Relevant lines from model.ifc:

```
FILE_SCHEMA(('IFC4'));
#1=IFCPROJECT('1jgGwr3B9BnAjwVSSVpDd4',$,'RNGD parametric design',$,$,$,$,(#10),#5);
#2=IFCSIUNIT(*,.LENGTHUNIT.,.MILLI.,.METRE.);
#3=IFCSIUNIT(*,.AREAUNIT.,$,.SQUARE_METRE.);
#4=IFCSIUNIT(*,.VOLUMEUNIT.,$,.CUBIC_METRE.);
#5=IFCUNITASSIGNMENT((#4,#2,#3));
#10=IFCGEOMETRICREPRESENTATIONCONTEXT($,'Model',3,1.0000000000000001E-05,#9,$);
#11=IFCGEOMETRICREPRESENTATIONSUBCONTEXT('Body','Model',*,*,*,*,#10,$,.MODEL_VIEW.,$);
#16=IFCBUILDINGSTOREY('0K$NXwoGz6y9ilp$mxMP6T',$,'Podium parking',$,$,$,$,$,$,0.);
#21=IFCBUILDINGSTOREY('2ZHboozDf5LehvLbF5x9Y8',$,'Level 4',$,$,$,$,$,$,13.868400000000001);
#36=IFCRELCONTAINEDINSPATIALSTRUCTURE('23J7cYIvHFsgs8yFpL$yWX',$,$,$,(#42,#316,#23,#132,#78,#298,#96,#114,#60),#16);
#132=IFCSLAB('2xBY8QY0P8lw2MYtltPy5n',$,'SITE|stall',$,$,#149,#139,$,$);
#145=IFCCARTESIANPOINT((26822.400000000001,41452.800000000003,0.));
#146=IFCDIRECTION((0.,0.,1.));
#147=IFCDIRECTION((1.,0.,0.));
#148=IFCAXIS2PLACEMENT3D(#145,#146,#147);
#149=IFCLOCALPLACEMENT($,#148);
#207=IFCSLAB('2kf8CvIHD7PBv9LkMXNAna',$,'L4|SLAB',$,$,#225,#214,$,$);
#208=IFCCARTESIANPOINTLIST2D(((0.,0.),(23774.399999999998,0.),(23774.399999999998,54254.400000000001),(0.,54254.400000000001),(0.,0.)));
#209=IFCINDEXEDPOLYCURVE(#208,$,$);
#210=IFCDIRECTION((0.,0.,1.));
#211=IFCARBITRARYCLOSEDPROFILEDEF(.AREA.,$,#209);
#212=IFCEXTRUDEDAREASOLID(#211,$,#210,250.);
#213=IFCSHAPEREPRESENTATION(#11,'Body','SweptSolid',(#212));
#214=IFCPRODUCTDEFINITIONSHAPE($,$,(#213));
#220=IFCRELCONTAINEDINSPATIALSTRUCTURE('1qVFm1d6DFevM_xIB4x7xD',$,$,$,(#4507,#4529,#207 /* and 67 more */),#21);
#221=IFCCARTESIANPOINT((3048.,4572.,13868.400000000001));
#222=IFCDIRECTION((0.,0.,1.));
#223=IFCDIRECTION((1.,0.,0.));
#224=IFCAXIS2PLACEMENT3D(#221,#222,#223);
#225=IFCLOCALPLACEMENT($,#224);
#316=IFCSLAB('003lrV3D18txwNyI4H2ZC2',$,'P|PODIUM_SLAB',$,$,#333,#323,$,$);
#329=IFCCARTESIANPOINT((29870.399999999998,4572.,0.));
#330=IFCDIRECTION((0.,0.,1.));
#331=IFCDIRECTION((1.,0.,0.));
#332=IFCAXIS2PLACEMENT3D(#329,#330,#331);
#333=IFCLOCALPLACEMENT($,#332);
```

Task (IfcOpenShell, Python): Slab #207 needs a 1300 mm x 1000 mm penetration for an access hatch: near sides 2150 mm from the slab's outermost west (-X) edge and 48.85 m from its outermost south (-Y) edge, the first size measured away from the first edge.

```python
import numpy as np
import ifcopenshell
import ifcopenshell.api.feature
import ifcopenshell.api.geometry
import ifcopenshell.api.root
import ifcopenshell.geom
import ifcopenshell.util.placement
import ifcopenshell.util.representation
import ifcopenshell.util.shape
import ifcopenshell.util.unit

model = ifcopenshell.open("model.ifc")
unit_scale = ifcopenshell.util.unit.calculate_unit_scale(model)
settings = ifcopenshell.geom.settings()


def volume(element):
    """Net volume in cubic metres, openings subtracted."""
    shape = ifcopenshell.geom.create_shape(settings, element)
    return ifcopenshell.util.shape.get_volume(shape.geometry)


slab = model.by_guid("2kf8CvIHD7PBv9LkMXNAna")
before = volume(slab)

# Extent in the slab's own axes, in metres. The edges named are its -X and -Y sides.
slab_shape = ifcopenshell.geom.create_shape(settings, slab)
vertices = ifcopenshell.util.shape.get_vertices(slab_shape.geometry)
x_min, y_min, bottom = vertices.min(axis=0)
top = vertices[:, 2].max()

opening = ifcopenshell.api.root.create_entity(model, ifc_class="IfcOpeningElement", name="Access hatch opening", predefined_type="OPENING")
context = ifcopenshell.util.representation.get_context(model, "Model", "Body", "MODEL_VIEW")
width, depth = 1.3, 1
outline = [(0.0, 0.0), (width, 0.0), (width, depth), (0.0, depth), (0.0, 0.0)]
# Overshoot both faces by 50 mm so the cut is clean.
shape = ifcopenshell.api.geometry.add_slab_representation(
    model, context=context, depth=top - bottom + 0.1, polyline=outline
)
ifcopenshell.api.geometry.assign_representation(model, product=opening, representation=shape)

matrix = ifcopenshell.util.placement.get_local_placement(slab.ObjectPlacement)
matrix[:, 3] = matrix @ np.append(np.array([x_min + 2.15, y_min + 48.85, bottom - 0.05]) / unit_scale, 1.0)
ifcopenshell.api.geometry.edit_object_placement(model, product=opening, matrix=matrix, is_si=False)
ifcopenshell.api.feature.add_feature(model, feature=opening, element=slab)

after = volume(slab)

print(f"slab volume {before:.3f} -> {after:.3f} m3")

model.write("model_updated.ifc")
```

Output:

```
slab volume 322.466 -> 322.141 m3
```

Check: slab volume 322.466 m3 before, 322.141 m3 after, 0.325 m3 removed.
